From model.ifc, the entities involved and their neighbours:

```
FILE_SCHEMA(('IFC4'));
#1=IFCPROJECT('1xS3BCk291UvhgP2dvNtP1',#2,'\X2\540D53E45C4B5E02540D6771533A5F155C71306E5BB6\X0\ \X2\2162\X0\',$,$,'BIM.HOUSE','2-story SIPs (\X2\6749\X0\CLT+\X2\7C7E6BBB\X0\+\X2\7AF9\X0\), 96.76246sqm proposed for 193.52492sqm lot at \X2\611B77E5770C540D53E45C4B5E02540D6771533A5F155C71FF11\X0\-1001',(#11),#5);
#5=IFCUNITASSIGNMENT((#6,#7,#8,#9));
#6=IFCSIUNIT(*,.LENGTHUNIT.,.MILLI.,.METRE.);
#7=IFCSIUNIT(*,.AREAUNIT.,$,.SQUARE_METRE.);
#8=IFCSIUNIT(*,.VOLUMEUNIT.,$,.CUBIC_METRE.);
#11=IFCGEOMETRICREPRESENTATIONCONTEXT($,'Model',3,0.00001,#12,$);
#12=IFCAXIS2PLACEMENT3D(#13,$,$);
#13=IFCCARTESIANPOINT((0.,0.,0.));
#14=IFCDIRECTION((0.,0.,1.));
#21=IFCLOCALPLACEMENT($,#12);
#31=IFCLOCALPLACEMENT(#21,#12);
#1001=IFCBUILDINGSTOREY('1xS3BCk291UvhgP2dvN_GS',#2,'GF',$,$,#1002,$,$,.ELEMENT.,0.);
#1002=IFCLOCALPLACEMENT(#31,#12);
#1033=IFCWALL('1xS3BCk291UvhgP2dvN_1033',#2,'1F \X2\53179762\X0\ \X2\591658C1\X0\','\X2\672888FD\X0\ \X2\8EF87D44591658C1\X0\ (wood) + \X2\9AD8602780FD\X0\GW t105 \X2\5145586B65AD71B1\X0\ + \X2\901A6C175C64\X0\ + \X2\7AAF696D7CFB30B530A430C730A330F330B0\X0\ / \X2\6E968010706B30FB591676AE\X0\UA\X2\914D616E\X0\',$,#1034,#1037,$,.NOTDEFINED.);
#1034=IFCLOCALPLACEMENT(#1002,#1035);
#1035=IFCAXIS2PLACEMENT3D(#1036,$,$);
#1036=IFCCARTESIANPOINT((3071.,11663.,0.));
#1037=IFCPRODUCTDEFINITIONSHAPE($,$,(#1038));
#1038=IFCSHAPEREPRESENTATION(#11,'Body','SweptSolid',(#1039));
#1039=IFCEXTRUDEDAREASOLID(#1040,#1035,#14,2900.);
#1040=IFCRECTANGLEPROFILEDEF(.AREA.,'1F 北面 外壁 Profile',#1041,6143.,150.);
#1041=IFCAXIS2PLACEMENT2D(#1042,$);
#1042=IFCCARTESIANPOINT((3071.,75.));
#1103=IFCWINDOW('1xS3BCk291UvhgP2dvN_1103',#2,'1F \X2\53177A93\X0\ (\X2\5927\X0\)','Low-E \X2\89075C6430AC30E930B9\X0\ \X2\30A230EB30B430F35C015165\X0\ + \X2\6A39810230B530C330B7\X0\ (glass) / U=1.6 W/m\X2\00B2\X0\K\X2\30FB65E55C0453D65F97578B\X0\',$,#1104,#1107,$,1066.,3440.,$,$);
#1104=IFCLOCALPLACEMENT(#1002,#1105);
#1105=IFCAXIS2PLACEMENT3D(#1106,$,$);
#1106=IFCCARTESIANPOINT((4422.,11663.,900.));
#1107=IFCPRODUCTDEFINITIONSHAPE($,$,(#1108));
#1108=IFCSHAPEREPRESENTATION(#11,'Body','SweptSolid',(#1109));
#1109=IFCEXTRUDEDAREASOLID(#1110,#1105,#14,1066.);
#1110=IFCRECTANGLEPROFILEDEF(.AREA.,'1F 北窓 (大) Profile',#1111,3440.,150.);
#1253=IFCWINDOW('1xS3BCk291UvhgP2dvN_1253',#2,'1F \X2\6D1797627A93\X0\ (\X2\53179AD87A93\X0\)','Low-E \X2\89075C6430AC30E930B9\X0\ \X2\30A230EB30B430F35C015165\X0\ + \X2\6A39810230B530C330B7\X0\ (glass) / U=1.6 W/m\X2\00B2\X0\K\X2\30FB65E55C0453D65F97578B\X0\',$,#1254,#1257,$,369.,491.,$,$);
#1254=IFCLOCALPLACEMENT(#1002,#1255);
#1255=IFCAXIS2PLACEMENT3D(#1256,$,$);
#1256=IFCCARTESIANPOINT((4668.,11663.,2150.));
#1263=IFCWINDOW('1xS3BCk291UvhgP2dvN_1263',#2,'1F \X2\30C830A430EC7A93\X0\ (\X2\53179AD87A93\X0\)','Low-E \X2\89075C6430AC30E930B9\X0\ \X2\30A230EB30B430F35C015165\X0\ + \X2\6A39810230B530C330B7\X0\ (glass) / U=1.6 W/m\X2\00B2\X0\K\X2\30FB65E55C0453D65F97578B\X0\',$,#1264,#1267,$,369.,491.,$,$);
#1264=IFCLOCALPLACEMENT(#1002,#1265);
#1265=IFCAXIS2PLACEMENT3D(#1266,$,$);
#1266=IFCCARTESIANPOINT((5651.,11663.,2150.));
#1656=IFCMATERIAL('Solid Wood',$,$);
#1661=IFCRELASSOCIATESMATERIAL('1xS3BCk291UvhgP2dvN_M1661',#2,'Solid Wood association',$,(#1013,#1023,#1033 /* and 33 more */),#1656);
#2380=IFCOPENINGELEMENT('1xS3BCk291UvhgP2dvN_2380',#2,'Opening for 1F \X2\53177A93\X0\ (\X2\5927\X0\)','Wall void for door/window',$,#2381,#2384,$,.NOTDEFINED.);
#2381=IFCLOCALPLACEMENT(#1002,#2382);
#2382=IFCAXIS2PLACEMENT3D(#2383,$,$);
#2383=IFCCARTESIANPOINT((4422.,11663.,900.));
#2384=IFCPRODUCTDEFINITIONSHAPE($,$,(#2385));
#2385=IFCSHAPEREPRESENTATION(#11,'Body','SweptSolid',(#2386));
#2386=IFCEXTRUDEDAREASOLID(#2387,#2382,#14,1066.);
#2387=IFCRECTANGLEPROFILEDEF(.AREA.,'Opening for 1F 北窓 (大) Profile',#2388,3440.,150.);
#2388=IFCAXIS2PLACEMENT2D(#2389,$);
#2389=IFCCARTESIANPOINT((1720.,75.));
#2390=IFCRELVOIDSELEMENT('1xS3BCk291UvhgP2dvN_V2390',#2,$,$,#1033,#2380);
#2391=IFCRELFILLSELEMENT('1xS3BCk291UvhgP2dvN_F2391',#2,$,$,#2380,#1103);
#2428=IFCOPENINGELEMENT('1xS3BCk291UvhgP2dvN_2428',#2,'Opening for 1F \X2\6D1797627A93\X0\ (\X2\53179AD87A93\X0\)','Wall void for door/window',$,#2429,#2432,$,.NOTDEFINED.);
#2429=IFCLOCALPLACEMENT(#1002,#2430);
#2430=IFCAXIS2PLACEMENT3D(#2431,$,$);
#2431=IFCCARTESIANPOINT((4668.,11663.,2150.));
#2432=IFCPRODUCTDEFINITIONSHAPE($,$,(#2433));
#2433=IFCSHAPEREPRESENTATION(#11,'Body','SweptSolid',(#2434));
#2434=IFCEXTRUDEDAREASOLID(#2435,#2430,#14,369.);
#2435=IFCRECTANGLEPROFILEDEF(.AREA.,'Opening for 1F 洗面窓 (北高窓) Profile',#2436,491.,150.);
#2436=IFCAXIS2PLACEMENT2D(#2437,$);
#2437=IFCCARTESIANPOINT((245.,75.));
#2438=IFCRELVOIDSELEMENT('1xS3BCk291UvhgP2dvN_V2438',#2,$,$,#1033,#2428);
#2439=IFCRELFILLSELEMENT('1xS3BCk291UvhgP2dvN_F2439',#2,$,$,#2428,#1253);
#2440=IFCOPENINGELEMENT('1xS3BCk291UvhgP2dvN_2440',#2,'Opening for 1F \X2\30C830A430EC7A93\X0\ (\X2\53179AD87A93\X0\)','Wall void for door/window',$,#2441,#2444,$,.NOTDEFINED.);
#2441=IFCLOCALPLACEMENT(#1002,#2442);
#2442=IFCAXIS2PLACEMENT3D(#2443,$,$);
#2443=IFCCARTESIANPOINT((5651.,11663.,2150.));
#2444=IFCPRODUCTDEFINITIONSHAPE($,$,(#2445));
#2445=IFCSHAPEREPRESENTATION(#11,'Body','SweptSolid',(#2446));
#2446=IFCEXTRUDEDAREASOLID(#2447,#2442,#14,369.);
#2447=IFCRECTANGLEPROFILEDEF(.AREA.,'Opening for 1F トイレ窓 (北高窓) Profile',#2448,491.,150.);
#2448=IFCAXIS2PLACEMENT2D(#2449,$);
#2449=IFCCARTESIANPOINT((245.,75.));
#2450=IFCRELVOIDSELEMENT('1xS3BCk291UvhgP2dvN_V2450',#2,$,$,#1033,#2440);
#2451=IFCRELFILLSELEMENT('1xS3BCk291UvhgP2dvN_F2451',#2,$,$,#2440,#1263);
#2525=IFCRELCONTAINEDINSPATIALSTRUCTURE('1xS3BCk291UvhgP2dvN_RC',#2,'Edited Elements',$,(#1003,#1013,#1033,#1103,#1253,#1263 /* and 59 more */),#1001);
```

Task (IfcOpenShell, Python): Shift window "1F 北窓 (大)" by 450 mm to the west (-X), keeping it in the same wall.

```python
import ifcopenshell
import ifcopenshell.api.geometry
import ifcopenshell.util.placement
import ifcopenshell.util.unit

model = ifcopenshell.open("model.ifc")
unit_scale = ifcopenshell.util.unit.calculate_unit_scale(model)

window = model.by_guid("1xS3BCk291UvhgP2dvN_1103")
opening = window.FillsVoids[0].RelatingOpeningElement
wall = opening.VoidsElements[0].RelatingBuildingElement

wall_matrix = ifcopenshell.util.placement.get_local_placement(wall.ObjectPlacement)
shift = wall_matrix[:3, 0] * -0.45 / unit_scale
before = ifcopenshell.util.placement.get_local_placement(window.ObjectPlacement)[:3, 3].copy()

# The window is not placed relative to its opening, so move both.
for product in (opening, window):
    matrix = ifcopenshell.util.placement.get_local_placement(product.ObjectPlacement)
    matrix[:3, 3] += shift
    ifcopenshell.api.geometry.edit_object_placement(model, product=product, matrix=matrix, is_si=False)

after = ifcopenshell.util.placement.get_local_placement(window.ObjectPlacement)[:3, 3]
print("window moved by", (after - before).round(3) + 0.0)

model.write("model_v2.ifc")
```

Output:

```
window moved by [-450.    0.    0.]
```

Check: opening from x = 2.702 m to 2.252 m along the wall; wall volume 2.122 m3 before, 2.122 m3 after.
